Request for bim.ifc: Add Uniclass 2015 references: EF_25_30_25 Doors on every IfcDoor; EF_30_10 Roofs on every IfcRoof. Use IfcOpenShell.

First a look at what the model holds.

```python
import ifcopenshell

model = ifcopenshell.open("bim.ifc")
print(model.schema)
print("classifications:", [c.Name for c in model.by_type("IfcClassification")])
for ifc_class in ("IfcDoor", "IfcRoof", "IfcStair", "IfcWall", "IfcWindow"):
    print(ifc_class, len(model.by_type(ifc_class)))
```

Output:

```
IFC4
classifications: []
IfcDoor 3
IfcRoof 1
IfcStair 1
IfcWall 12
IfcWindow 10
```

```python
import ifcopenshell
import ifcopenshell.api.classification

model = ifcopenshell.open("bim.ifc")

system = ifcopenshell.api.classification.add_classification(model, classification="Uniclass 2015")

codes = {
    "IfcDoor": ("EF_25_30_25", "Doors"),
    "IfcRoof": ("EF_30_10", "Roofs"),
}
for ifc_class, (code, name) in codes.items():
    products = model.by_type(ifc_class)
    ifcopenshell.api.classification.add_reference(
        model, products=products, classification=system, identification=code, name=name
    )
    print(code, len(products))

model.write("bim_edited.ifc")
```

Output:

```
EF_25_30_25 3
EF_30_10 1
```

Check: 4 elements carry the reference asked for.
